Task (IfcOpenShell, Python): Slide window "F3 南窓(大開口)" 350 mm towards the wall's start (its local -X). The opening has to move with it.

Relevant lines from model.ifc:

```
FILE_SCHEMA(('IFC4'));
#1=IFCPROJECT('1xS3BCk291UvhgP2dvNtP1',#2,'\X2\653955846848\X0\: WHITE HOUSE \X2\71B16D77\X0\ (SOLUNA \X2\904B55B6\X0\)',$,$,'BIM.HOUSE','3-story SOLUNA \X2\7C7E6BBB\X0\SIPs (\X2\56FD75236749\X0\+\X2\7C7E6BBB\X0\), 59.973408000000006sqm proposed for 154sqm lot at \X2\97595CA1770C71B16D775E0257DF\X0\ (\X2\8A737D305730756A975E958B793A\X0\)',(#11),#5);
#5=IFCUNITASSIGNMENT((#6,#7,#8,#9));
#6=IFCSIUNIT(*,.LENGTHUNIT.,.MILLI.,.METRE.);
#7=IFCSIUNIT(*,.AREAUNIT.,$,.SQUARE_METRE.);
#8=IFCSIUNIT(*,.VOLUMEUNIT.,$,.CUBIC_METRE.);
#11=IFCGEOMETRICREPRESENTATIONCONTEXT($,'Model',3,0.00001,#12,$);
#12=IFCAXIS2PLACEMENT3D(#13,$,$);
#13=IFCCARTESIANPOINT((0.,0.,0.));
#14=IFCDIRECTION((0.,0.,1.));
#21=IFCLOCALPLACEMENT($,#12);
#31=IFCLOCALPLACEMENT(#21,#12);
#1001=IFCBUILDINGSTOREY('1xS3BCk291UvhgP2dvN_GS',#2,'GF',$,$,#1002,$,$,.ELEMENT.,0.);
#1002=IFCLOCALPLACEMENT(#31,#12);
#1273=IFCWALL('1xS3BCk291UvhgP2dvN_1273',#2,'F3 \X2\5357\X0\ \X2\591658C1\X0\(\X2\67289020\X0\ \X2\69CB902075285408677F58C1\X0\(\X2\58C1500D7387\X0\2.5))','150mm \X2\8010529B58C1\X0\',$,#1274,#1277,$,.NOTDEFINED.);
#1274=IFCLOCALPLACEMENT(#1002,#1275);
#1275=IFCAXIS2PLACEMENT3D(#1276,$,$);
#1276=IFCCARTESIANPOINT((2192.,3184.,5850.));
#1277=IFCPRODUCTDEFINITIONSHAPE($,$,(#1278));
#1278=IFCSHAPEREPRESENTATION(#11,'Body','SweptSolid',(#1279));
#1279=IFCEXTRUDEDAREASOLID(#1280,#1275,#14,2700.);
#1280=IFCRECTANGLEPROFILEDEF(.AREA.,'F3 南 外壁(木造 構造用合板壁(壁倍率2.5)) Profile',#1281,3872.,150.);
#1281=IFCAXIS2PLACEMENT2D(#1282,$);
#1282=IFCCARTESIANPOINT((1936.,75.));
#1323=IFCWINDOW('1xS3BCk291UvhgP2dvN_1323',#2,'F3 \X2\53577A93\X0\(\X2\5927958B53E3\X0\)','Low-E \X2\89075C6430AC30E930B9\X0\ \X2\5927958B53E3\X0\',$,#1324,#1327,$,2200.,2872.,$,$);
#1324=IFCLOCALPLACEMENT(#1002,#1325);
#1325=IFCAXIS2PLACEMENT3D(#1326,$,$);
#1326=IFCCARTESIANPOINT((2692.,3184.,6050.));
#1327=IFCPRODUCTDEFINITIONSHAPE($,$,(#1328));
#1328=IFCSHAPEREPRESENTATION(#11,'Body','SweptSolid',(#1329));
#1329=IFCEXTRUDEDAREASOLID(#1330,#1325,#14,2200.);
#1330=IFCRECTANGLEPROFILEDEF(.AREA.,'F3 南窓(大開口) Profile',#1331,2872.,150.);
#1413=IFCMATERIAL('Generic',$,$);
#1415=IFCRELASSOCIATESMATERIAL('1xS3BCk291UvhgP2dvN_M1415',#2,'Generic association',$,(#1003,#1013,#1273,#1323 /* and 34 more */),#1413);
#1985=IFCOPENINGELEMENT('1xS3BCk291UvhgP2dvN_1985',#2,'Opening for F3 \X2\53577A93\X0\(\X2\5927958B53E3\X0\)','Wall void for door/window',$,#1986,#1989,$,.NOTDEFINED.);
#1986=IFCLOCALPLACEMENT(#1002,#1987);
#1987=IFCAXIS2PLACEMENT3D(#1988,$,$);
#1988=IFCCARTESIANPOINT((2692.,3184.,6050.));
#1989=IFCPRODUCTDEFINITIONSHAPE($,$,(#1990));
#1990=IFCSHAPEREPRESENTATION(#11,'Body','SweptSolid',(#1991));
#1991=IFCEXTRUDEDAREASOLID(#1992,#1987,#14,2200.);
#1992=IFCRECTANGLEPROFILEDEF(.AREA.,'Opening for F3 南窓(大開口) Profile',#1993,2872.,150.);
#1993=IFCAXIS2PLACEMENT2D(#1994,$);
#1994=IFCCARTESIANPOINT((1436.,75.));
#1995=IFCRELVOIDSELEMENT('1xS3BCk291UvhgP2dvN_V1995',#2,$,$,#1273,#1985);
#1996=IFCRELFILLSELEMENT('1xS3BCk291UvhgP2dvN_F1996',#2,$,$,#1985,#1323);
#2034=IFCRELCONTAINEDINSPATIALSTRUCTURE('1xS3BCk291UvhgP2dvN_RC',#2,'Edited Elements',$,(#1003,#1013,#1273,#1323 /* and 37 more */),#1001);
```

```python
import ifcopenshell
import ifcopenshell.api.geometry
import ifcopenshell.util.placement

model = ifcopenshell.open("model.ifc")

window = model.by_guid("1xS3BCk291UvhgP2dvN_1323")
opening = window.FillsVoids[0].RelatingOpeningElement
wall = opening.VoidsElements[0].RelatingBuildingElement

wall_matrix = ifcopenshell.util.placement.get_local_placement(wall.ObjectPlacement)
shift = wall_matrix[:3, 0] * -350.0
before = ifcopenshell.util.placement.get_local_placement(window.ObjectPlacement)[:3, 3].copy()

# The window is not placed relative to its opening, so move both.
for product in (opening, window):
    matrix = ifcopenshell.util.placement.get_local_placement(product.ObjectPlacement)
    matrix[:3, 3] += shift
    ifcopenshell.api.geometry.edit_object_placement(model, product=product, matrix=matrix, is_si=False)

after = ifcopenshell.util.placement.get_local_placement(window.ObjectPlacement)[:3, 3]
print("window moved by", (after - before).round(3) + 0.0)

model.write("model_rev.ifc")
```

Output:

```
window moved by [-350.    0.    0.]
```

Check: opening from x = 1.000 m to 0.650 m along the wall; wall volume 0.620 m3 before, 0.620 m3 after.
